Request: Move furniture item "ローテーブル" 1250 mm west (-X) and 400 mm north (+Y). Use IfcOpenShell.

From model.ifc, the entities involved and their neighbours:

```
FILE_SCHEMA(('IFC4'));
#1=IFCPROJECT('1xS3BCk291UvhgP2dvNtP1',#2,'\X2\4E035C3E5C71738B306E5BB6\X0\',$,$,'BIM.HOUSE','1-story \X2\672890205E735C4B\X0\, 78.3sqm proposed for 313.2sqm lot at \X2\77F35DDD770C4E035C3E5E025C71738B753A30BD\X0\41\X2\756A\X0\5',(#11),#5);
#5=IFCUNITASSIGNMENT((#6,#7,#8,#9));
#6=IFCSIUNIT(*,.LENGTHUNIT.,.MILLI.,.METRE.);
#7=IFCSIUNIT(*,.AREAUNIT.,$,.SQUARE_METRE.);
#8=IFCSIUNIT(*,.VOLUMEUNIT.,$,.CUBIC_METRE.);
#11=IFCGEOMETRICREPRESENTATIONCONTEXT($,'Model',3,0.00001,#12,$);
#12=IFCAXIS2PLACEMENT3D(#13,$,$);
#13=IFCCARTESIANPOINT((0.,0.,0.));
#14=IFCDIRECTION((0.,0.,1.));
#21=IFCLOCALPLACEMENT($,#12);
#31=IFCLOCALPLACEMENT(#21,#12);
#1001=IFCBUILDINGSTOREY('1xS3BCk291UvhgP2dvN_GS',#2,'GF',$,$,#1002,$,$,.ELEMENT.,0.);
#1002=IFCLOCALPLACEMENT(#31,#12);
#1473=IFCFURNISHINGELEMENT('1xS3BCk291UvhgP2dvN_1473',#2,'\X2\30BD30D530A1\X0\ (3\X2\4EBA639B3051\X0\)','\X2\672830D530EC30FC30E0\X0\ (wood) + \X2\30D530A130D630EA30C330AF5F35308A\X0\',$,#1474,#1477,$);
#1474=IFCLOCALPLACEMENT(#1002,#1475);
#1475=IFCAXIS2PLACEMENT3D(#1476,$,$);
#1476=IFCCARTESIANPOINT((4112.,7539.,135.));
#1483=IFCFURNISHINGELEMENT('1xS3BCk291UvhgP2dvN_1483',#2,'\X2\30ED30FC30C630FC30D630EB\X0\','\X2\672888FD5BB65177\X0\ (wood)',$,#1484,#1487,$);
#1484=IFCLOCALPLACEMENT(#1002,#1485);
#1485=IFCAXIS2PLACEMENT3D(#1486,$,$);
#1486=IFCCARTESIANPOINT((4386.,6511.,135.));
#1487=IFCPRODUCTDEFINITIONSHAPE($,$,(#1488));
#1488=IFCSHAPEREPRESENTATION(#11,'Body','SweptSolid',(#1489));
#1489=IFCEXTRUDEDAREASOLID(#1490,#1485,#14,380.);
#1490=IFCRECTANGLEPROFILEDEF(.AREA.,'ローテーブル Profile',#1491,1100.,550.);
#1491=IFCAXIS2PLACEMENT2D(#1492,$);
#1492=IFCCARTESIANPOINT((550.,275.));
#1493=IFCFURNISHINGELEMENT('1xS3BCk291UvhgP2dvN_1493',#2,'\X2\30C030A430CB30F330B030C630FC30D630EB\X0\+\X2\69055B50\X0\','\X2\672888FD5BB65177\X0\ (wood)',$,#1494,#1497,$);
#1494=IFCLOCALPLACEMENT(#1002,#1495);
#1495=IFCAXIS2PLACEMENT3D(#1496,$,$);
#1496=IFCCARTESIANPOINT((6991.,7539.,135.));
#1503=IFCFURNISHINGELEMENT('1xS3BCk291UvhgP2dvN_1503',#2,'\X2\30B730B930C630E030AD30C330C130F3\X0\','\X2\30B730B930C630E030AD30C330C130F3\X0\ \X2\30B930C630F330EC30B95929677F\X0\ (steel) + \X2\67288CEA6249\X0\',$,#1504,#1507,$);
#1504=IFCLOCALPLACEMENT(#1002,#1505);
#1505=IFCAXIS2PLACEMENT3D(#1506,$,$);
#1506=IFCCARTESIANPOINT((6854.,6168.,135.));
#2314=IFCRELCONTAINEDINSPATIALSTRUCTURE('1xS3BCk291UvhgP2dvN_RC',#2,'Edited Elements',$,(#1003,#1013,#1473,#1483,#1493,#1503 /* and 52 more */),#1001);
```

```python
import ifcopenshell
import ifcopenshell.api.geometry
import ifcopenshell.util.placement
import ifcopenshell.util.unit

model = ifcopenshell.open("model.ifc")
unit_scale = ifcopenshell.util.unit.calculate_unit_scale(model)

item = model.by_id(1483)
matrix = ifcopenshell.util.placement.get_local_placement(item.ObjectPlacement)
matrix[0, 3] -= 1.25 / unit_scale
matrix[1, 3] += 0.4 / unit_scale
ifcopenshell.api.geometry.edit_object_placement(model, product=item, matrix=matrix, is_si=False)

print(ifcopenshell.util.placement.get_local_placement(item.ObjectPlacement).round(3) + 0.0)

model.write("model_updated.ifc")
```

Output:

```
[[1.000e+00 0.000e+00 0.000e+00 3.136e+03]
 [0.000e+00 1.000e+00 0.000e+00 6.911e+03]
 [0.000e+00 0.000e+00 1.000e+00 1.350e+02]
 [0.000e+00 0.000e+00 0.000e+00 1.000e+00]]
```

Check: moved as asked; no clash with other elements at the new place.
